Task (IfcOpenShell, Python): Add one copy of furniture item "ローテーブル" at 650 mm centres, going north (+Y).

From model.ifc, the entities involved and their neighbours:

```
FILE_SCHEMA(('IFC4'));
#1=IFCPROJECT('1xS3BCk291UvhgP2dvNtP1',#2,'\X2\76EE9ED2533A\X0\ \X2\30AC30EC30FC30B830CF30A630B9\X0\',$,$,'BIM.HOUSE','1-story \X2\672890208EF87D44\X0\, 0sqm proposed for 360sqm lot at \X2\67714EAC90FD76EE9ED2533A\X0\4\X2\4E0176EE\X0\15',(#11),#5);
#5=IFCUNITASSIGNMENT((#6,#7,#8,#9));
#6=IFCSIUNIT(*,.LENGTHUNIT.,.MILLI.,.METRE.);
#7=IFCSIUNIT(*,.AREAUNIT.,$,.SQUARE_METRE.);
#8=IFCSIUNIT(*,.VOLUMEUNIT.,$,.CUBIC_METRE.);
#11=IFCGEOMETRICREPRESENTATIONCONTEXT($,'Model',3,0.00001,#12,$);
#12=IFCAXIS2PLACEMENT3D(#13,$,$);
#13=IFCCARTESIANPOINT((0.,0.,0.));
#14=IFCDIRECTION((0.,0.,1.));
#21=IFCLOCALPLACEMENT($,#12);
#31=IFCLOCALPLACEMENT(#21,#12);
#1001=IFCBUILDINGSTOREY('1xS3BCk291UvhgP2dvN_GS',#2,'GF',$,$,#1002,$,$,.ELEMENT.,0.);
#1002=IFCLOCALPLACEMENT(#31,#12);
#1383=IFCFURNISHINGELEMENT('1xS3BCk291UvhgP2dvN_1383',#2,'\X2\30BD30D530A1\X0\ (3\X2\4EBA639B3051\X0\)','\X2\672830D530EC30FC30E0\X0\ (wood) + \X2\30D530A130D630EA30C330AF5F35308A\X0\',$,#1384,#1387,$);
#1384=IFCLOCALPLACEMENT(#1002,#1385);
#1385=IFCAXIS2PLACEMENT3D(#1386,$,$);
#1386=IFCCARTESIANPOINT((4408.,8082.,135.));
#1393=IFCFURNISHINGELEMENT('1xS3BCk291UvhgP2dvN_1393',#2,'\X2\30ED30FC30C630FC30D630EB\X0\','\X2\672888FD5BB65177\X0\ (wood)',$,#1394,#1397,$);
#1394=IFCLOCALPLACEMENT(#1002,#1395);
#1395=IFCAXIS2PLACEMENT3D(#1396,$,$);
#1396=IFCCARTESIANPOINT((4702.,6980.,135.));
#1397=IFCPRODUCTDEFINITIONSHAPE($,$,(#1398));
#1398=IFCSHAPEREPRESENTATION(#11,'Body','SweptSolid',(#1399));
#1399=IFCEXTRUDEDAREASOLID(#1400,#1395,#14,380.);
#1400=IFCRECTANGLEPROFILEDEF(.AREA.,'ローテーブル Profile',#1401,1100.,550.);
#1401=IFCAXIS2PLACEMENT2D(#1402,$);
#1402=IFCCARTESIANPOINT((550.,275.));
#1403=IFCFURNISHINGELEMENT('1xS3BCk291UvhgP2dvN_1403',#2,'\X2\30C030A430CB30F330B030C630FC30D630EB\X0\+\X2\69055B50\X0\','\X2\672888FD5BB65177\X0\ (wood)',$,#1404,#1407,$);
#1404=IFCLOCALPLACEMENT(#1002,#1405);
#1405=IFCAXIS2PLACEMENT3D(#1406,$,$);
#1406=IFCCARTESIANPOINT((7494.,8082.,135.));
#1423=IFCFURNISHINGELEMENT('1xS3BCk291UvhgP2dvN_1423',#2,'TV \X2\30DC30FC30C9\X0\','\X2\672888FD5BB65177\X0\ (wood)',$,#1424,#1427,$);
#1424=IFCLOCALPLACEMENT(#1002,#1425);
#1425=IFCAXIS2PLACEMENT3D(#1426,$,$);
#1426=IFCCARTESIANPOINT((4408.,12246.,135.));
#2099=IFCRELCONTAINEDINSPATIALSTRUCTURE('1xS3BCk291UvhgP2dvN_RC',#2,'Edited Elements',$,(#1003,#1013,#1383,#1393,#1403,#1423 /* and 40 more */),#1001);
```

```python
import numpy as np
import ifcopenshell
import ifcopenshell.api.geometry
import ifcopenshell.api.root
import ifcopenshell.util.element
import ifcopenshell.util.placement

model = ifcopenshell.open("model.ifc")


def reuse_history(source, copy):
    """copy_class also copies each property set's owner history, people and application; keep the originals."""
    for rel in copy.IsDefinedBy:
        if rel.is_a("IfcRelDefinesByProperties") and (history := rel.RelatingPropertyDefinition.OwnerHistory):
            rel.RelatingPropertyDefinition.OwnerHistory = source.OwnerHistory
            ifcopenshell.util.element.remove_deep2(model, history)


source = model.by_guid("1xS3BCk291UvhgP2dvN_1393")
base = ifcopenshell.util.placement.get_local_placement(source.ObjectPlacement)
step = np.array([0.0, 1.0, 0.0]) * 650.0

for i in range(1, 2):
    copy = ifcopenshell.api.root.copy_class(model, product=source)
    copy.Representation = ifcopenshell.util.element.copy_deep(
        model, source.Representation, exclude=["IfcGeometricRepresentationContext", "IfcRepresentationMap"]
    )
    reuse_history(source, copy)
    matrix = base.copy()
    matrix[:3, 3] += i * step
    print("added at", matrix[:3, 3].round(3) + 0.0)
    ifcopenshell.api.geometry.edit_object_placement(model, product=copy, matrix=matrix, is_si=False)

model.write("model_v2.ifc")
```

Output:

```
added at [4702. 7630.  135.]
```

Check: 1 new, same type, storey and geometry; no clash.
